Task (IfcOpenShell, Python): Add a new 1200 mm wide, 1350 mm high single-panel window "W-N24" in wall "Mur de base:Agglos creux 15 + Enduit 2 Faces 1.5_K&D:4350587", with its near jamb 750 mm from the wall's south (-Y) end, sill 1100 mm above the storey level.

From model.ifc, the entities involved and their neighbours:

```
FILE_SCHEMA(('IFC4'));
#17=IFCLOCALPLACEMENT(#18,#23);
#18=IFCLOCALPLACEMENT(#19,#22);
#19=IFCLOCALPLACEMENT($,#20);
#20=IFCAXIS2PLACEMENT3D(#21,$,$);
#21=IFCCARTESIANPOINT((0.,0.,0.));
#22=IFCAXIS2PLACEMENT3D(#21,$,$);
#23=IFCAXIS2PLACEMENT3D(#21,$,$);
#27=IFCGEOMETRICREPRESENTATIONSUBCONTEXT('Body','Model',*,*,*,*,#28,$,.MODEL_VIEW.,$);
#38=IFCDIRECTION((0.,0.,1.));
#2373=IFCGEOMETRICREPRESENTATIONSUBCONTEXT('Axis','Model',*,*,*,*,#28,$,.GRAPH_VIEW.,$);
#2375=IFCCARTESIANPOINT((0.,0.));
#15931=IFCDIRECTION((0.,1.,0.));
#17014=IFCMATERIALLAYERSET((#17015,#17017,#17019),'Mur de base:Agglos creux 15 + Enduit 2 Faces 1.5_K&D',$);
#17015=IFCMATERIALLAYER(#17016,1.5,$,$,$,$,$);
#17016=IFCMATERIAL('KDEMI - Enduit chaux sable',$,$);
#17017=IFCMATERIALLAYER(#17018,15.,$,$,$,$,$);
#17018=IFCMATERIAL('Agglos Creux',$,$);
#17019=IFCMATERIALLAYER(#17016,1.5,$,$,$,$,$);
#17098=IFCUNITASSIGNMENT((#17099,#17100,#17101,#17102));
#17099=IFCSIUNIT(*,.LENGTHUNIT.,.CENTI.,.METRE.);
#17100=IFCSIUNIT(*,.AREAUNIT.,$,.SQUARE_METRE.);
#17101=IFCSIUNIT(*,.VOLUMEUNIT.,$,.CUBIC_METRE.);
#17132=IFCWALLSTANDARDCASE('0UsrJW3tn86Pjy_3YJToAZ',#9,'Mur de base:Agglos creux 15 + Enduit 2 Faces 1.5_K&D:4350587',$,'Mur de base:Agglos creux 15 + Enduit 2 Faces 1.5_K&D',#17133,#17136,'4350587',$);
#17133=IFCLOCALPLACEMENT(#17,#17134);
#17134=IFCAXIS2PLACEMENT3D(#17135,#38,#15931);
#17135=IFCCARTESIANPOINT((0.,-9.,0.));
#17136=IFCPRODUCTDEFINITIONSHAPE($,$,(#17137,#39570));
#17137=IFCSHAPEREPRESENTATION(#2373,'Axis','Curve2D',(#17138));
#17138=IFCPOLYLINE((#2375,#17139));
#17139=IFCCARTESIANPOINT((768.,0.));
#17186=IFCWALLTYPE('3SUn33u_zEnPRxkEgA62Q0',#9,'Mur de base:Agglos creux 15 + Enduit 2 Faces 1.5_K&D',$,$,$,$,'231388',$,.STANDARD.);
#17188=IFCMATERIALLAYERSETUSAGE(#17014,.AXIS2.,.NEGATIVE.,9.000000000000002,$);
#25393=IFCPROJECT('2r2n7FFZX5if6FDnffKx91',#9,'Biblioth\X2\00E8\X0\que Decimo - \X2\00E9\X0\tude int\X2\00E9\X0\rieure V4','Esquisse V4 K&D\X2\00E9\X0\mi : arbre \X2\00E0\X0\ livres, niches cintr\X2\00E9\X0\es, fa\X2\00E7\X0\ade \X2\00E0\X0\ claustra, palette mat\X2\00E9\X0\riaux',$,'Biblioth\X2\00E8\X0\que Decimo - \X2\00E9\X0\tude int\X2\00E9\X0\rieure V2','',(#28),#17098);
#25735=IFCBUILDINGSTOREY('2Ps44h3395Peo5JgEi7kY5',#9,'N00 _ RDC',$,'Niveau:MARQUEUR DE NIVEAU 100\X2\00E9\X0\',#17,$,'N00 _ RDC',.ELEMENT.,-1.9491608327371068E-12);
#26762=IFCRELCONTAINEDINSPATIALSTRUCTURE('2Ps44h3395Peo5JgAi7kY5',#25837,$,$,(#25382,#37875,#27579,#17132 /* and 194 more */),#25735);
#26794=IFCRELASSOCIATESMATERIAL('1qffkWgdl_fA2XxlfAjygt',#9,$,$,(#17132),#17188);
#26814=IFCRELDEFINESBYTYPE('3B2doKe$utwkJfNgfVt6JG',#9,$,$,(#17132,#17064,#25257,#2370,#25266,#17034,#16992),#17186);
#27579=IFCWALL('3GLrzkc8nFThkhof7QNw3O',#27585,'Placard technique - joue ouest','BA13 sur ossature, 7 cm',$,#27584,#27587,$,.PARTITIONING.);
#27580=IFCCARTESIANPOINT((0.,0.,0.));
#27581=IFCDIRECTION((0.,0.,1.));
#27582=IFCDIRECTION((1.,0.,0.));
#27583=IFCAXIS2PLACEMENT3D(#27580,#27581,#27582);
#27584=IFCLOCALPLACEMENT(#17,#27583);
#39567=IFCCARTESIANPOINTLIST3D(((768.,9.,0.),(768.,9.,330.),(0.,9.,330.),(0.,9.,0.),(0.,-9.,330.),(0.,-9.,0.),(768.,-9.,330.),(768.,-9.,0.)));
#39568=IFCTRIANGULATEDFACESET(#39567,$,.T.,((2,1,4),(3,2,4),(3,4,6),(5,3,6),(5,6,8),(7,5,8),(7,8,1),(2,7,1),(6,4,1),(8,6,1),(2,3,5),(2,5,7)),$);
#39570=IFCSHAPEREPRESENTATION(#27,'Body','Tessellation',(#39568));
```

```python
import numpy as np
import ifcopenshell
import ifcopenshell.api.feature
import ifcopenshell.api.geometry
import ifcopenshell.api.root
import ifcopenshell.api.spatial
import ifcopenshell.geom
import ifcopenshell.util.element
import ifcopenshell.util.placement
import ifcopenshell.util.representation
import ifcopenshell.util.shape
import ifcopenshell.util.unit

model = ifcopenshell.open("model.ifc")
unit_scale = ifcopenshell.util.unit.calculate_unit_scale(model)
settings = ifcopenshell.geom.settings()


def volume(element):
    """Net volume in cubic metres, openings subtracted."""
    shape = ifcopenshell.geom.create_shape(settings, element)
    return ifcopenshell.util.shape.get_volume(shape.geometry)


wall = model.by_id(17132)
storey = ifcopenshell.util.element.get_container(wall, ifc_class="IfcBuildingStorey")
context = ifcopenshell.util.representation.get_context(model, "Model", "Body", "MODEL_VIEW")
before = volume(wall)

width, height, from_end, sill = 1.2, 1.35, 0.75, 1.1  # metres

# The wall runs along its own X axis, and the end named is its -X end.
wall_shape = ifcopenshell.geom.create_shape(settings, wall)
x, y, z = ifcopenshell.util.shape.get_vertices(wall_shape.geometry).T
start = x.min() + from_end
face, thickness = float(y.min()), float(y.max() - y.min())
wall_matrix = ifcopenshell.util.placement.get_local_placement(wall.ObjectPlacement)
level = ifcopenshell.util.placement.get_local_placement(storey.ObjectPlacement)[2, 3]


def in_wall(x, y):
    """Placement at x, y metres in the wall's axes, at sill height."""
    matrix = wall_matrix.copy()
    matrix[:, 3] = wall_matrix @ np.array([x / unit_scale, y / unit_scale, 0.0, 1.0])
    matrix[2, 3] = level + sill / unit_scale
    return matrix


# Opening: a box that overshoots both wall faces by 50 mm.
opening = ifcopenshell.api.root.create_entity(model, ifc_class="IfcOpeningElement", predefined_type="OPENING")
box = ifcopenshell.api.geometry.add_wall_representation(
    model, context=context, length=width, height=height, thickness=thickness + 0.1
)
ifcopenshell.api.geometry.assign_representation(model, product=opening, representation=box)
ifcopenshell.api.geometry.edit_object_placement(model, product=opening, matrix=in_wall(start, face - 0.05), is_si=False)
ifcopenshell.api.feature.add_feature(model, feature=opening, element=wall)

window = ifcopenshell.api.root.create_entity(model, ifc_class="IfcWindow", name="W-N24", predefined_type="WINDOW")
window.OverallWidth, window.OverallHeight = width / unit_scale, height / unit_scale
window.PartitioningType = "SINGLE_PANEL"
body = ifcopenshell.api.geometry.add_window_representation(
    model,
    context=context,
    overall_width=window.OverallWidth,
    overall_height=window.OverallHeight,
    partition_type="SINGLE_PANEL",
)
ifcopenshell.api.geometry.assign_representation(model, product=window, representation=body)
ifcopenshell.api.spatial.assign_container(model, products=[window], relating_structure=storey)
ifcopenshell.api.feature.add_filling(model, opening=opening, element=window)

# Centre the window in the wall's thickness.
ifcopenshell.api.geometry.edit_object_placement(model, product=window, matrix=in_wall(start, face), is_si=False)
window_shape = ifcopenshell.geom.create_shape(settings, window)
depth = ifcopenshell.util.shape.get_vertices(window_shape.geometry)[:, 1]
offset = face + thickness / 2 - (depth.min() + depth.max()) / 2
ifcopenshell.api.geometry.edit_object_placement(model, product=window, matrix=in_wall(start, offset), is_si=False)

after = volume(wall)

print(f"wall volume {before:.3f} -> {after:.3f} m3")

model.write("model_v2.ifc")
```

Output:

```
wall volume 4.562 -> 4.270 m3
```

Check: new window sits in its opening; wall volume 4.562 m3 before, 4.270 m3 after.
